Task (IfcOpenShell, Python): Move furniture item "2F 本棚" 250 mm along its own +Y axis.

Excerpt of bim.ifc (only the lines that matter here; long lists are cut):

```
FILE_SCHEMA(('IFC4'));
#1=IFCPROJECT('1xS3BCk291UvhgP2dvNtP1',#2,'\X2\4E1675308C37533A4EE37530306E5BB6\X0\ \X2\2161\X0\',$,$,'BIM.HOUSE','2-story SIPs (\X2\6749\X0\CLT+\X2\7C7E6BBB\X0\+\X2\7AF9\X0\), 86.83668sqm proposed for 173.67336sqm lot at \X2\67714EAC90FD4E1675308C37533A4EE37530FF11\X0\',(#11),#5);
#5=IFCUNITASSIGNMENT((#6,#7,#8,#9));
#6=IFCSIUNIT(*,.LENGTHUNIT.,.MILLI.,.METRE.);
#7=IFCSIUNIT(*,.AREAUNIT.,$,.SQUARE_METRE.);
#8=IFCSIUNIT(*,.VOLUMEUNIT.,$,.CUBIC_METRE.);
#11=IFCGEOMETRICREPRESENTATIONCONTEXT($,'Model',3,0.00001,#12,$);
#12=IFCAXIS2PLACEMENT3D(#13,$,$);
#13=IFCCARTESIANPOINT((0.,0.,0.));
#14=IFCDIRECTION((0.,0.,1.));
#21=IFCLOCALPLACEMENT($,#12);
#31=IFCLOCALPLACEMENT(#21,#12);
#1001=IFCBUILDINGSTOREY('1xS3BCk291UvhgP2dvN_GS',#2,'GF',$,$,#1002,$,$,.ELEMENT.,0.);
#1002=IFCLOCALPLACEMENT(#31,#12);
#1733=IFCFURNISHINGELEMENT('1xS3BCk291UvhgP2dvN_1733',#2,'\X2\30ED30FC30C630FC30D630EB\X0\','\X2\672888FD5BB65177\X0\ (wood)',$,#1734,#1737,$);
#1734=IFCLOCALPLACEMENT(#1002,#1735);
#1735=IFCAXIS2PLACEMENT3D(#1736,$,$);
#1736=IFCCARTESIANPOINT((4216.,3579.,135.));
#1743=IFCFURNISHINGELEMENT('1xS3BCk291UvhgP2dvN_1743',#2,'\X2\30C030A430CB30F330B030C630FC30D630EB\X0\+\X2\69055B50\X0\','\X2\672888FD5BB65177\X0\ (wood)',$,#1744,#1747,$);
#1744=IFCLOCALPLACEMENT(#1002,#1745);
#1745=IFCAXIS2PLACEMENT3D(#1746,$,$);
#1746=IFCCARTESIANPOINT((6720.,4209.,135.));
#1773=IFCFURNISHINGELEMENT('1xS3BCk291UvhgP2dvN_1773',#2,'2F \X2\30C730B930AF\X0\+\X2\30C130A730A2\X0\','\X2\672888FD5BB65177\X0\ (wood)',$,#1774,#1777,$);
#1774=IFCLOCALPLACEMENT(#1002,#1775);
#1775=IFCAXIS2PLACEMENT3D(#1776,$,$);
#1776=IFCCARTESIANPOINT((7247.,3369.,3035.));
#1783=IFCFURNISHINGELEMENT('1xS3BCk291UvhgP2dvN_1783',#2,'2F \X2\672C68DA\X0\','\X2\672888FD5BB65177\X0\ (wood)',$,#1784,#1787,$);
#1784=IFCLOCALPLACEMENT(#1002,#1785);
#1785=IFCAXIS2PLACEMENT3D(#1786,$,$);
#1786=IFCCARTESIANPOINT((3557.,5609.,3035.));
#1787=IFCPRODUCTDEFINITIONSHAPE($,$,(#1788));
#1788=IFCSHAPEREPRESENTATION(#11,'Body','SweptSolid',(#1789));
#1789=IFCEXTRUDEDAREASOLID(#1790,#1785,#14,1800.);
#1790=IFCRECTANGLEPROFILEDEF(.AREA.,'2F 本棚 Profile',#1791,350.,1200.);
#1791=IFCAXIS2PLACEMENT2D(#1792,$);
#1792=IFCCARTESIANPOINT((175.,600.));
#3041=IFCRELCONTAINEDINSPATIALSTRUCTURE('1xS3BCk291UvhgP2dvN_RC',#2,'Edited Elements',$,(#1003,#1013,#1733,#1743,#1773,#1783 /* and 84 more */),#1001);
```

```python
import ifcopenshell
import ifcopenshell.api.geometry
import ifcopenshell.util.placement
import ifcopenshell.util.unit

model = ifcopenshell.open("bim.ifc")
unit_scale = ifcopenshell.util.unit.calculate_unit_scale(model)

item = model.by_id(1783)
matrix = ifcopenshell.util.placement.get_local_placement(item.ObjectPlacement)
matrix[:3, 3] += matrix[:3, 1] * 0.25 / unit_scale
ifcopenshell.api.geometry.edit_object_placement(model, product=item, matrix=matrix, is_si=False)

print(ifcopenshell.util.placement.get_local_placement(item.ObjectPlacement).round(3) + 0.0)

model.write("bim-out.ifc")
```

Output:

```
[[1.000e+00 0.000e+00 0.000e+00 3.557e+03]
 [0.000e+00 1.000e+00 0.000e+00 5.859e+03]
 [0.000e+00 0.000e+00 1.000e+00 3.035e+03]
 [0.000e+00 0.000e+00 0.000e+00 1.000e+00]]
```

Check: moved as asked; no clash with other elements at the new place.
